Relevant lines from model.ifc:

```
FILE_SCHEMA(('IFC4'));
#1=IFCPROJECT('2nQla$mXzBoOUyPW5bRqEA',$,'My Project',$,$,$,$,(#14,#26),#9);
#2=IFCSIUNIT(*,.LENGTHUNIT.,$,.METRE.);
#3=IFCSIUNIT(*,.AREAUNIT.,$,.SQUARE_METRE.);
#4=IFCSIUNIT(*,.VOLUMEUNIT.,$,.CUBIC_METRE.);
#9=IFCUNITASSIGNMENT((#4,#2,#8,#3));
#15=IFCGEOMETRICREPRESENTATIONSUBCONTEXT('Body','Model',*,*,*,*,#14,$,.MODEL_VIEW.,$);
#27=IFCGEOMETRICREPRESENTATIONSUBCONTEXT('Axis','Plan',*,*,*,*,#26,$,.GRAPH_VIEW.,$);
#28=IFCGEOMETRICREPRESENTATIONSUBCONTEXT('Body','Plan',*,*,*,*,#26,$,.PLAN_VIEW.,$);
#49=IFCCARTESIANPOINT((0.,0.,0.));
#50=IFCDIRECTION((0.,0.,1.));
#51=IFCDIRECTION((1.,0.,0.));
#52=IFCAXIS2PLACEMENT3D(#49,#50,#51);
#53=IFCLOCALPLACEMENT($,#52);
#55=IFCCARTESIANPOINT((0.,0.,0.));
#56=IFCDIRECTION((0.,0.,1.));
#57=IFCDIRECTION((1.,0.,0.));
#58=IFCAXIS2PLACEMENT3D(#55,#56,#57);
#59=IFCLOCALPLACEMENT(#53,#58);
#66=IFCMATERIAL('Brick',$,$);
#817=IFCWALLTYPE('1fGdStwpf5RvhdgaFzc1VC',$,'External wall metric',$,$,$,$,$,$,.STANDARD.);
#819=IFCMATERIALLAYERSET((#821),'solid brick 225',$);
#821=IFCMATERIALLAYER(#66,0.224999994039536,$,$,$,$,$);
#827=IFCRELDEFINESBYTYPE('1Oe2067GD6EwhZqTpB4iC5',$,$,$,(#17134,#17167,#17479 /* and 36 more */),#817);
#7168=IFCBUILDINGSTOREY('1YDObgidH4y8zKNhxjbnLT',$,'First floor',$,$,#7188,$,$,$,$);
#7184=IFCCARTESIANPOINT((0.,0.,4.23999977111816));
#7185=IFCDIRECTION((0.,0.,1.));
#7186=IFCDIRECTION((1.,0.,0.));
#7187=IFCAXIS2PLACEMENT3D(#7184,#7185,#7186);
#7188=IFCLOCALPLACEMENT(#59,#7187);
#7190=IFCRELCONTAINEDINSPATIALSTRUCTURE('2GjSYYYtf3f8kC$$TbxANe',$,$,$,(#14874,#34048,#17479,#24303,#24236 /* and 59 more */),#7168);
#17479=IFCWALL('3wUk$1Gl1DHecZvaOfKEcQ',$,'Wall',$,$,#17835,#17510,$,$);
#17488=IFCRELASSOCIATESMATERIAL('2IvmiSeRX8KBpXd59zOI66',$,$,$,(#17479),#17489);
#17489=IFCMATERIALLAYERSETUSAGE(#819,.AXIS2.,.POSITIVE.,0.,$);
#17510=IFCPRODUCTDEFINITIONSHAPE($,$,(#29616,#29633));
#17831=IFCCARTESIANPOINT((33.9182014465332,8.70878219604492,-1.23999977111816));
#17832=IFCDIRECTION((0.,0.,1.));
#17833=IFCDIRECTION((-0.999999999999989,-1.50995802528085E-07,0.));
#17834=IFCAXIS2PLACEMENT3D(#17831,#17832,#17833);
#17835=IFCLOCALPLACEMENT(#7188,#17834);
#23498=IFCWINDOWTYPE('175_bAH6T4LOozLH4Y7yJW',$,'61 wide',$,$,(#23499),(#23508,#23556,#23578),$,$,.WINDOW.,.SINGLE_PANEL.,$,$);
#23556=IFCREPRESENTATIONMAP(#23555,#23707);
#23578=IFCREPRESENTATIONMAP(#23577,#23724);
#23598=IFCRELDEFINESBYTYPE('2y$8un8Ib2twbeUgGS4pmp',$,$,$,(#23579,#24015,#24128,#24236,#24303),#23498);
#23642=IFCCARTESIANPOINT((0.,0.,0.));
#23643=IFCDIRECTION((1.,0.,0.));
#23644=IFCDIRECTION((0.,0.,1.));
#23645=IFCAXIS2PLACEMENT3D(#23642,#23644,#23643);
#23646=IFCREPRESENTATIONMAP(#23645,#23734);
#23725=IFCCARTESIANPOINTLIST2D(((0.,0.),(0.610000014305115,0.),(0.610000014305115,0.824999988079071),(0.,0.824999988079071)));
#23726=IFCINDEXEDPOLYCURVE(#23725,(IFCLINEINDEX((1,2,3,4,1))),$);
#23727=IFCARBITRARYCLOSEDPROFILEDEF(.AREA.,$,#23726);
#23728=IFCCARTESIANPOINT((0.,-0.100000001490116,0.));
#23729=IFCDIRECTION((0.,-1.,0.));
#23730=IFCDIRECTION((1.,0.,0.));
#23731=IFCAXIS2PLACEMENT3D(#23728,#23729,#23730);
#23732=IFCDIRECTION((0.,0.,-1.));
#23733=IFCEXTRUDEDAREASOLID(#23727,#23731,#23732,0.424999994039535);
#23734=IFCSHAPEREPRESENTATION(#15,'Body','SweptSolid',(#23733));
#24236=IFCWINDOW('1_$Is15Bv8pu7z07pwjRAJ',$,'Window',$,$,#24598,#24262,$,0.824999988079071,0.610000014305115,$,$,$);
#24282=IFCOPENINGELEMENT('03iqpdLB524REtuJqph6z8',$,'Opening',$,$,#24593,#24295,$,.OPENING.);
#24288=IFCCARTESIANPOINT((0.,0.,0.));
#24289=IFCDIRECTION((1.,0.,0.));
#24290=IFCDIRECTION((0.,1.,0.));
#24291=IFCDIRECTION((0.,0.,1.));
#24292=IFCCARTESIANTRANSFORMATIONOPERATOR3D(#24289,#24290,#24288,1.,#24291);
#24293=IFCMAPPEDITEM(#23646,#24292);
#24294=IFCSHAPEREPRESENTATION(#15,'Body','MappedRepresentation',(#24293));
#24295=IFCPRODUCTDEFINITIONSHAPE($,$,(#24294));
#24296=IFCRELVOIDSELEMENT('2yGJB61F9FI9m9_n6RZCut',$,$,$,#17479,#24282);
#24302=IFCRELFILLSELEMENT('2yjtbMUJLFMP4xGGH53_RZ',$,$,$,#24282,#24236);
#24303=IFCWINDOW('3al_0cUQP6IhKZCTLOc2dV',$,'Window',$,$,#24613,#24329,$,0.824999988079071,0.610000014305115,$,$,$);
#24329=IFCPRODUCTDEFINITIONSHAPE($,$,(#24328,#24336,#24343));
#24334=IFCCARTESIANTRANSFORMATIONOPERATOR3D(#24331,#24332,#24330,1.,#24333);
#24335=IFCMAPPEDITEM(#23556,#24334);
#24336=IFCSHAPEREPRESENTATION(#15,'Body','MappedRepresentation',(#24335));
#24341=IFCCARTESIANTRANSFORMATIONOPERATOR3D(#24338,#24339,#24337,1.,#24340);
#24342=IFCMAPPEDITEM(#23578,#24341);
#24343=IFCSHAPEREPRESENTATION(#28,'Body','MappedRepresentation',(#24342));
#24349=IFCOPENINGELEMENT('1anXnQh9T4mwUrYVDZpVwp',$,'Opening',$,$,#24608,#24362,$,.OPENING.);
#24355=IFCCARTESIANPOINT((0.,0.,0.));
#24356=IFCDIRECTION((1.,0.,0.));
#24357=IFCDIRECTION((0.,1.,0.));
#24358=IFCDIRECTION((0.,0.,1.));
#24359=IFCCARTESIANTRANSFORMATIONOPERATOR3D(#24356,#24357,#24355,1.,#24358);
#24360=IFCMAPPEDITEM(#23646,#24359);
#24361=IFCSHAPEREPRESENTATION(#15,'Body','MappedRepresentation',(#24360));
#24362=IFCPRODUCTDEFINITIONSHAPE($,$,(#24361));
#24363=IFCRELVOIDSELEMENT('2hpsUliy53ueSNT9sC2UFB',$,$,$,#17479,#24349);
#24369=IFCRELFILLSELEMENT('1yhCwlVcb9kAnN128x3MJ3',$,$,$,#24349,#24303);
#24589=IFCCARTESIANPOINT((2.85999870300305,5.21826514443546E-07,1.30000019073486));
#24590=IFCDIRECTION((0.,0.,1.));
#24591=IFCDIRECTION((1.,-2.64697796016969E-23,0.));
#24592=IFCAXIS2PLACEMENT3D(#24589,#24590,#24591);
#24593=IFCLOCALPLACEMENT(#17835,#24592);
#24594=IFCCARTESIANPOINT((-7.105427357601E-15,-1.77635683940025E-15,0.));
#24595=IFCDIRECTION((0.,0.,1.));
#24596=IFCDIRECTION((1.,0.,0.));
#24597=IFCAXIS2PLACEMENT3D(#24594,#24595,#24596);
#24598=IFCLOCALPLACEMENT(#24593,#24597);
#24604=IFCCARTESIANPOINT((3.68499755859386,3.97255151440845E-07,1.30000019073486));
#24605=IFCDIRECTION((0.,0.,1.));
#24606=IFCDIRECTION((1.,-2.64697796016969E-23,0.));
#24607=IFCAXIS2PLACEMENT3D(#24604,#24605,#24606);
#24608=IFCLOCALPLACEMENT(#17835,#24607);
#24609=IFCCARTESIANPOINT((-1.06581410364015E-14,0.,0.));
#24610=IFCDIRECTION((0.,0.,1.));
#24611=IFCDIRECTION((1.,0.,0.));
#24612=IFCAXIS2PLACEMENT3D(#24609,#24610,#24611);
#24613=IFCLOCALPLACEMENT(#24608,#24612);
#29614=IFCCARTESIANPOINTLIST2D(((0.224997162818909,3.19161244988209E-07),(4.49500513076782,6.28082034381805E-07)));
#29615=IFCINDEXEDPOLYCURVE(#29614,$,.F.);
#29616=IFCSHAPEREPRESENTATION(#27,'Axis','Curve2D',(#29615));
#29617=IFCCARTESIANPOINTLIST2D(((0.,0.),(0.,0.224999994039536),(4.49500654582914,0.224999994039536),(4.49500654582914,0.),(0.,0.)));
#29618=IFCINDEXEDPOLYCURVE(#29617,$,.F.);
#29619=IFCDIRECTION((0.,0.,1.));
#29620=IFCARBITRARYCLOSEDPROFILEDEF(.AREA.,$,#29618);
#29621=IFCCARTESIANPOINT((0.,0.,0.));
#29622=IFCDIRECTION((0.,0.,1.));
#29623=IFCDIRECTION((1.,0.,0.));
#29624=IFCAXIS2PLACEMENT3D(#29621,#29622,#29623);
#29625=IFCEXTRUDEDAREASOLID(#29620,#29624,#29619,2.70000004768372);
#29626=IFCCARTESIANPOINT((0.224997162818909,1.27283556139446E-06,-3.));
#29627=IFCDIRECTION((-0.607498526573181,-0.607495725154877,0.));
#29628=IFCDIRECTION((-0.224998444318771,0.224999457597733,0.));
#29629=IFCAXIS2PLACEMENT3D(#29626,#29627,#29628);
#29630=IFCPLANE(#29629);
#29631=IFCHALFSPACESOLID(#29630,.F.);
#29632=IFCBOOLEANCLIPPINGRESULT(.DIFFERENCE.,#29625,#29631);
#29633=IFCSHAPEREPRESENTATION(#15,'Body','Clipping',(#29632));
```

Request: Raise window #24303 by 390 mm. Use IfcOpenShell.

```python
import numpy as np
import ifcopenshell
import ifcopenshell.api.geometry
import ifcopenshell.util.placement
import ifcopenshell.util.unit

model = ifcopenshell.open("model.ifc")
unit_scale = ifcopenshell.util.unit.calculate_unit_scale(model)

window = model.by_guid("3al_0cUQP6IhKZCTLOc2dV")
opening = window.FillsVoids[0].RelatingOpeningElement
dz = 0.39

shift = np.array([0.0, 0.0, dz])
# The window is placed relative to its opening, so it follows when the opening moves.
matrix = ifcopenshell.util.placement.get_local_placement(opening.ObjectPlacement)
matrix[:3, 3] += shift
ifcopenshell.api.geometry.edit_object_placement(
    model, product=opening, matrix=matrix, is_si=False, should_transform_children=True
)

print(f"moved by {dz * unit_scale:+.3f} m")

model.write("model_rev.ifc")
```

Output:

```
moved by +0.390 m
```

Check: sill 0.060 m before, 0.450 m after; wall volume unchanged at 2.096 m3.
